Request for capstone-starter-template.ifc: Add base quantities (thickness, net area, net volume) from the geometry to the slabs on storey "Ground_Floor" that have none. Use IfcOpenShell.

First a look at what the model holds.

```python
import ifcopenshell
import ifcopenshell.util.element
import ifcopenshell.util.unit

model = ifcopenshell.open("capstone-starter-template.ifc")
print(model.schema)
for unit_type in ("LENGTHUNIT", "AREAUNIT", "VOLUMEUNIT"):
    print(unit_type, ifcopenshell.util.unit.calculate_unit_scale(model, unit_type))
storey = next(s for s in model.by_type("IfcBuildingStorey") if s.Name == "Ground_Floor")
slabs = [e for e in ifcopenshell.util.element.get_decomposition(storey) if e.is_a("IfcSlab")]
for e in sorted(slabs, key=lambda e: e.id()):
    print(e.id(), e.is_a(), e.Name, list(ifcopenshell.util.element.get_psets(e, qtos_only=True)), sep=" | ")
```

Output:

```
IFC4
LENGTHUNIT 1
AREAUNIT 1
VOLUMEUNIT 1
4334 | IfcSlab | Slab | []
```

```python
import ifcopenshell
import ifcopenshell.api.pset
import ifcopenshell.geom
import ifcopenshell.util.element
import ifcopenshell.util.shape
import ifcopenshell.util.unit

model = ifcopenshell.open("capstone-starter-template.ifc")
unit_scale = ifcopenshell.util.unit.calculate_unit_scale(model)
area_scale = ifcopenshell.util.unit.calculate_unit_scale(model, "AREAUNIT")
volume_scale = ifcopenshell.util.unit.calculate_unit_scale(model, "VOLUMEUNIT")
settings = ifcopenshell.geom.settings()

storey = next(s for s in model.by_type("IfcBuildingStorey") if s.Name == "Ground_Floor")
slabs = [e for e in ifcopenshell.util.element.get_decomposition(storey) if e.is_a("IfcSlab")]

for e in sorted(slabs, key=lambda e: e.id()):
    if ifcopenshell.util.element.get_psets(e, qtos_only=True, should_inherit=False):
        continue
    # Geometry comes back in metres, in the element's own axes.
    shape = ifcopenshell.geom.create_shape(settings, e)
    values = {
        "Width": ifcopenshell.util.shape.get_z(shape.geometry) / unit_scale,
        "NetArea": ifcopenshell.util.shape.get_footprint_area(shape.geometry) / area_scale,
        "NetVolume": ifcopenshell.util.shape.get_volume(shape.geometry) / volume_scale,
    }
    qto = ifcopenshell.api.pset.add_qto(model, product=e, name="Qto_SlabBaseQuantities")
    ifcopenshell.api.pset.edit_qto(model, qto=qto, properties=values)
    print(e.id(), {k: round(v, 3) for k, v in values.items()})

model.write("capstone-starter-template_edited.ifc")
```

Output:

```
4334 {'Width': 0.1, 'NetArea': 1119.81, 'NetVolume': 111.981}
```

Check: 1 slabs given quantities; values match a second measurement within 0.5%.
